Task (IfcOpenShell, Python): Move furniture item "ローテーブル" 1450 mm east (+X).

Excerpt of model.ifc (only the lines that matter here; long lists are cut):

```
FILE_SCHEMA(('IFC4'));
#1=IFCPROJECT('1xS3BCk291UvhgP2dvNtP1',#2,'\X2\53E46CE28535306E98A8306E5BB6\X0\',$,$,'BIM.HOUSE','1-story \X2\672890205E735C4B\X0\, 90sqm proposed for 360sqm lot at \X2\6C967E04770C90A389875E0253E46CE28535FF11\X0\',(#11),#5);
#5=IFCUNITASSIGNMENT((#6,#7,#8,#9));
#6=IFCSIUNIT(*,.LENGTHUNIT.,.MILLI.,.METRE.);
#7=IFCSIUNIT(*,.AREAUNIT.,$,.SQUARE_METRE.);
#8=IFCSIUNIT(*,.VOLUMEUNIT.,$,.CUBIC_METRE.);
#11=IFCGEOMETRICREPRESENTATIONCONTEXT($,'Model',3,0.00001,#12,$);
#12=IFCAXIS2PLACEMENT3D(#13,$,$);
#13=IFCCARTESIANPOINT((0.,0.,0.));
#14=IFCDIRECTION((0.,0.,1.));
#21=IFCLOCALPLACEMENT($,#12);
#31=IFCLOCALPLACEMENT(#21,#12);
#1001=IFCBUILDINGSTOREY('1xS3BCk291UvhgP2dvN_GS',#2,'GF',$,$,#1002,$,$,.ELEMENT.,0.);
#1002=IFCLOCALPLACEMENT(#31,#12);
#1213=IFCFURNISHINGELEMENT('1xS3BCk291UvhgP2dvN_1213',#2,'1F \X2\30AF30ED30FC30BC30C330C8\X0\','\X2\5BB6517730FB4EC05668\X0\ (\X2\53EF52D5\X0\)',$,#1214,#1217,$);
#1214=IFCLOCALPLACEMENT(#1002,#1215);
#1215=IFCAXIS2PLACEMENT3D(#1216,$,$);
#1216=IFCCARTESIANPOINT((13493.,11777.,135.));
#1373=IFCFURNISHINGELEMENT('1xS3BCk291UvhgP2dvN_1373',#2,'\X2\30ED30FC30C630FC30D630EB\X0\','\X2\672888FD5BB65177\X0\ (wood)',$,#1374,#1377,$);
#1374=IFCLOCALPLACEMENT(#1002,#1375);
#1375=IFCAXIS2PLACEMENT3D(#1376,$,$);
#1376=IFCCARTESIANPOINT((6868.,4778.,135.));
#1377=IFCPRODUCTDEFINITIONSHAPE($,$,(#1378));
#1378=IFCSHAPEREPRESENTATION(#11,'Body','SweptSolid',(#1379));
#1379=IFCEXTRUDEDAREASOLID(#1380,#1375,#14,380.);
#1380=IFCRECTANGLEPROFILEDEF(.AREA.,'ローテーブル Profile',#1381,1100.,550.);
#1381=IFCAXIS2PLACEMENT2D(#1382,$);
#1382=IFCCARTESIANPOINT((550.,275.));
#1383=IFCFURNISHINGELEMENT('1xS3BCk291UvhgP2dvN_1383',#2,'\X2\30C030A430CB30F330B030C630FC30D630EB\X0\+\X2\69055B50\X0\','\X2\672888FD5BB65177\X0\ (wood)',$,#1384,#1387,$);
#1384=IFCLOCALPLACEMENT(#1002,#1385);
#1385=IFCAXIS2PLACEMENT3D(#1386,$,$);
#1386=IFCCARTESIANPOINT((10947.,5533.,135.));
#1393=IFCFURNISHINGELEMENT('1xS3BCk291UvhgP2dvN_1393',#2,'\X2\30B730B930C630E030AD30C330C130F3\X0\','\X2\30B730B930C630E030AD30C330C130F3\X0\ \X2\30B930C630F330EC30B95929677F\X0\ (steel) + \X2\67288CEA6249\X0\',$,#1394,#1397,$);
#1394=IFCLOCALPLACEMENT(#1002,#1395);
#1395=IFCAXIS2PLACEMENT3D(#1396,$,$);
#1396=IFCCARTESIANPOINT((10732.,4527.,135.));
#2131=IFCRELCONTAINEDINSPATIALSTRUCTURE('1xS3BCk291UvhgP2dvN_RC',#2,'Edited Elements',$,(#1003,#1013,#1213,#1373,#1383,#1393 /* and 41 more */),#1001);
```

```python
import ifcopenshell
import ifcopenshell.api.geometry
import ifcopenshell.util.placement
import ifcopenshell.util.unit

model = ifcopenshell.open("model.ifc")
unit_scale = ifcopenshell.util.unit.calculate_unit_scale(model)

item = model.by_guid("1xS3BCk291UvhgP2dvN_1373")
matrix = ifcopenshell.util.placement.get_local_placement(item.ObjectPlacement)
matrix[0, 3] += 1.45 / unit_scale
ifcopenshell.api.geometry.edit_object_placement(model, product=item, matrix=matrix, is_si=False)

print(ifcopenshell.util.placement.get_local_placement(item.ObjectPlacement).round(3) + 0.0)

model.write("model_v2.ifc")
```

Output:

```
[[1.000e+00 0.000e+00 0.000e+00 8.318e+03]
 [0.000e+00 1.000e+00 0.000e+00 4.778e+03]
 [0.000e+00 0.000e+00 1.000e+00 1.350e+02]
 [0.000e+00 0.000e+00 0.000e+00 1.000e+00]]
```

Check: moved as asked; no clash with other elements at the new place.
